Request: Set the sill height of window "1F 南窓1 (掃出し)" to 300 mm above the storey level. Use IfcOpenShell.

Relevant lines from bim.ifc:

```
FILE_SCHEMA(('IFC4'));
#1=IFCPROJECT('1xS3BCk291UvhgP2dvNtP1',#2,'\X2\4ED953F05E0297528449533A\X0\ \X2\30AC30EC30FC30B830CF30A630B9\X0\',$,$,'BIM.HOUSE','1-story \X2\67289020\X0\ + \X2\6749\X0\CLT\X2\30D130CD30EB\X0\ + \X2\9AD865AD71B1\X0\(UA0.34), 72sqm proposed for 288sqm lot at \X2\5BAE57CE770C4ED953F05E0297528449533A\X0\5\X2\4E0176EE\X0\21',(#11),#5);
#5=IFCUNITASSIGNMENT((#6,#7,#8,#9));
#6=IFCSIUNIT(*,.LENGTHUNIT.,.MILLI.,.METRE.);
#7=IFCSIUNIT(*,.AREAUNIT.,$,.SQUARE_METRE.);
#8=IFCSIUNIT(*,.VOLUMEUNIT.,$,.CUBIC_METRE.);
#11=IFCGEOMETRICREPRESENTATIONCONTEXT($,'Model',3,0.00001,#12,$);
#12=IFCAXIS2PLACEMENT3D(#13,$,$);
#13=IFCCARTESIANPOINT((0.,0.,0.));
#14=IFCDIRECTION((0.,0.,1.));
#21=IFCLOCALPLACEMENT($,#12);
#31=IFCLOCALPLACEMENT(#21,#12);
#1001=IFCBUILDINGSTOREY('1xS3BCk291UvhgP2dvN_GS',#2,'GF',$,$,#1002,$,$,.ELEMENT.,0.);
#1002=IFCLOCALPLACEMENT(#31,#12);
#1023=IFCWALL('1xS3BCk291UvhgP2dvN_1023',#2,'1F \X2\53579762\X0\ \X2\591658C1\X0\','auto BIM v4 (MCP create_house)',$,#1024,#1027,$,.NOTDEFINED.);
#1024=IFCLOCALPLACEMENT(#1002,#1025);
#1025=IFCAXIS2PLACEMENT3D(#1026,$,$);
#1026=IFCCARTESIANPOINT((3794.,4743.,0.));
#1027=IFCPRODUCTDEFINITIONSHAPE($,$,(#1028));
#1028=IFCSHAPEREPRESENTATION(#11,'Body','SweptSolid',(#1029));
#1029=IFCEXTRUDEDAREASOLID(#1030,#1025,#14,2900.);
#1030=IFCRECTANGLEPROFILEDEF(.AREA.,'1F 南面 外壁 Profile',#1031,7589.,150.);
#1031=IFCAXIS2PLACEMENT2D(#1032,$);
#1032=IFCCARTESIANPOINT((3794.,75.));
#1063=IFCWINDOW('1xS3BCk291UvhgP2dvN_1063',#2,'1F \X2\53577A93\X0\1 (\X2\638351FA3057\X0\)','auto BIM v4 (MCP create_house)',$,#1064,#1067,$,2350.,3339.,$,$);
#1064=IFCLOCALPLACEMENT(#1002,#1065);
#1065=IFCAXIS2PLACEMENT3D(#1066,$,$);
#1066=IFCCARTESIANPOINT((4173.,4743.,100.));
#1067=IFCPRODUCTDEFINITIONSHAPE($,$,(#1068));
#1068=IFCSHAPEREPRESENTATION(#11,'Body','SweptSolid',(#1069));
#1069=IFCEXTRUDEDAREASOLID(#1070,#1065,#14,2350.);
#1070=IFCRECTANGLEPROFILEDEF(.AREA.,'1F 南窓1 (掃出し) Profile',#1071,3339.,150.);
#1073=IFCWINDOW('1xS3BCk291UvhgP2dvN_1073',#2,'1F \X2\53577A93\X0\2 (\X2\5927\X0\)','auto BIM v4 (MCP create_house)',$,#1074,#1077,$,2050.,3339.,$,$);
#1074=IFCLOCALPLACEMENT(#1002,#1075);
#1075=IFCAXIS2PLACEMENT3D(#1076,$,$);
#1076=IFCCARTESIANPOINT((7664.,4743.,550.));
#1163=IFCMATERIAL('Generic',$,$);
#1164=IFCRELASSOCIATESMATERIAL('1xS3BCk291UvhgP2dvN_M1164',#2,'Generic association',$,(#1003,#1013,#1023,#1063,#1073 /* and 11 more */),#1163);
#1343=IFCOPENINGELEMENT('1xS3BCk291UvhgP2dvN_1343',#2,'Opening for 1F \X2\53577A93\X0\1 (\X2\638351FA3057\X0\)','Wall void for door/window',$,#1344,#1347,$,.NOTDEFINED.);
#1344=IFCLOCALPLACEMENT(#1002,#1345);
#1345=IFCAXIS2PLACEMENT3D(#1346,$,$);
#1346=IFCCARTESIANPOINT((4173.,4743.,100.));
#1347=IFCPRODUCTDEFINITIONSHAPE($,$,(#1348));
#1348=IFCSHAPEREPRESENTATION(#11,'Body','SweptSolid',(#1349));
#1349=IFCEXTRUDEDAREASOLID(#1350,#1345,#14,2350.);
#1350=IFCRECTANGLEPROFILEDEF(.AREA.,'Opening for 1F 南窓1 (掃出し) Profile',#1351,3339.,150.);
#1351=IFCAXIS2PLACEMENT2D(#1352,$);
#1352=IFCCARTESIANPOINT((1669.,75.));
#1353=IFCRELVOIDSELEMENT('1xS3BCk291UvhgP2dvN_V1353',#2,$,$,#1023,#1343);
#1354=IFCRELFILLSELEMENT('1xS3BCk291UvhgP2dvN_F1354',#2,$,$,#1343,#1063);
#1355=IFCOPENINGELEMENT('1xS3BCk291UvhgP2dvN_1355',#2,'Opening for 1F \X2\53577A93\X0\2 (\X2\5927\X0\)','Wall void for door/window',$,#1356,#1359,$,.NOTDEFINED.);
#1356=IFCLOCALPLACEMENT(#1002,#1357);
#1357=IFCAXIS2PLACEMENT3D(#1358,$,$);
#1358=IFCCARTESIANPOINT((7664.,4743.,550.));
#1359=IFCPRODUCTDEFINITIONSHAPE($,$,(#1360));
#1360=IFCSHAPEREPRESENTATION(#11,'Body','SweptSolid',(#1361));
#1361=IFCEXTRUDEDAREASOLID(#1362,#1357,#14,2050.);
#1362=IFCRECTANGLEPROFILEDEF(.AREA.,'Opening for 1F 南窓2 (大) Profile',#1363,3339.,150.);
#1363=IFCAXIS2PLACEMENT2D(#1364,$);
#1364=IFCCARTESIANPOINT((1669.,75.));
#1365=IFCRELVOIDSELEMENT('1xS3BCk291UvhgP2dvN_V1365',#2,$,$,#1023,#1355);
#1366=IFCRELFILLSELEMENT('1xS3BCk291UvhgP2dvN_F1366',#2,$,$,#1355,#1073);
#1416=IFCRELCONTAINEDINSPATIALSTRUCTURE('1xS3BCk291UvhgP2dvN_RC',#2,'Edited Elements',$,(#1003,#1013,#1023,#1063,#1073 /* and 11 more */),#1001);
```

```python
import numpy as np
import ifcopenshell
import ifcopenshell.api.geometry
import ifcopenshell.geom
import ifcopenshell.util.element
import ifcopenshell.util.placement
import ifcopenshell.util.shape
import ifcopenshell.util.unit

model = ifcopenshell.open("bim.ifc")
unit_scale = ifcopenshell.util.unit.calculate_unit_scale(model)

window = model.by_guid("1xS3BCk291UvhgP2dvN_1063")
opening = window.FillsVoids[0].RelatingOpeningElement
storey = ifcopenshell.util.element.get_container(window, ifc_class="IfcBuildingStorey")
level = ifcopenshell.util.placement.get_local_placement(storey.ObjectPlacement)[2, 3]

# The opening's origin need not be at the sill, so measure its lowest point.
shape = ifcopenshell.geom.create_shape(ifcopenshell.geom.settings(), opening)
bottom = ifcopenshell.util.shape.get_shape_bottom_elevation(shape, shape.geometry) / unit_scale
dz = level + 300.0 - bottom

shift = np.array([0.0, 0.0, dz])
# The window is not placed relative to its opening, so move both.
for product in (opening, window):
    matrix = ifcopenshell.util.placement.get_local_placement(product.ObjectPlacement)
    matrix[:3, 3] += shift
    ifcopenshell.api.geometry.edit_object_placement(model, product=product, matrix=matrix, is_si=False)

print(f"moved by {dz * unit_scale:+.3f} m")

model.write("bim_rev.ifc")
```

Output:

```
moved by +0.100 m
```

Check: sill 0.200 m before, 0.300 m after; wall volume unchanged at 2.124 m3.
